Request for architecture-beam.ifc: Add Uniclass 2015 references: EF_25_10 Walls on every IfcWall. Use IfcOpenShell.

First a look at what the model holds.

```python
import ifcopenshell

model = ifcopenshell.open("architecture-beam.ifc")
print(model.schema)
print("classifications:", [c.Name for c in model.by_type("IfcClassification")])
for ifc_class in ("IfcDoor", "IfcRoof", "IfcStair", "IfcWall", "IfcWindow"):
    print(ifc_class, len(model.by_type(ifc_class)))
```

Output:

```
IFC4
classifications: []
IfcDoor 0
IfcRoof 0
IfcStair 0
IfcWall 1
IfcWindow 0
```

```python
import ifcopenshell
import ifcopenshell.api.classification

model = ifcopenshell.open("architecture-beam.ifc")

system = ifcopenshell.api.classification.add_classification(model, classification="Uniclass 2015")

codes = {
    "IfcWall": ("EF_25_10", "Walls"),
}
for ifc_class, (code, name) in codes.items():
    products = model.by_type(ifc_class)
    ifcopenshell.api.classification.add_reference(
        model, products=products, classification=system, identification=code, name=name
    )
    print(code, len(products))

model.write("architecture-beam_edited.ifc")
```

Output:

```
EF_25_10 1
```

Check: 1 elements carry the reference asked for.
